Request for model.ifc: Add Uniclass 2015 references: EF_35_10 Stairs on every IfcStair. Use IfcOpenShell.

First a look at what the model holds.

```python
import ifcopenshell

model = ifcopenshell.open("model.ifc")
print(model.schema)
print("classifications:", [c.Name for c in model.by_type("IfcClassification")])
for ifc_class in ("IfcDoor", "IfcRoof", "IfcStair", "IfcWall", "IfcWindow"):
    print(ifc_class, len(model.by_type(ifc_class)))
```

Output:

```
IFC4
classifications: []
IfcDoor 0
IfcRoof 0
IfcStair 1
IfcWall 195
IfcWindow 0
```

```python
import ifcopenshell
import ifcopenshell.api.classification

model = ifcopenshell.open("model.ifc")

system = ifcopenshell.api.classification.add_classification(model, classification="Uniclass 2015")

codes = {
    "IfcStair": ("EF_35_10", "Stairs"),
}
for ifc_class, (code, name) in codes.items():
    products = model.by_type(ifc_class)
    ifcopenshell.api.classification.add_reference(
        model, products=products, classification=system, identification=code, name=name
    )
    print(code, len(products))

model.write("model_v2.ifc")
```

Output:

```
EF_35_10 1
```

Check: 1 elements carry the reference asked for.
